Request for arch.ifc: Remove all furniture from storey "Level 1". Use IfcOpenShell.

First a look at what the model holds.

```python
import ifcopenshell
import ifcopenshell.util.element

model = ifcopenshell.open("arch.ifc")
print(model.schema)
storey = next(s for s in model.by_type("IfcBuildingStorey") if s.Name == "Level 1")
furniture = [e for e in ifcopenshell.util.element.get_decomposition(storey) if e.is_a("IfcFurnishingElement")]
seen = {}
for e in furniture:
    element_type = ifcopenshell.util.element.get_type(e)
    name = element_type.Name if element_type not in (None, e) else None
    seen[name] = seen.get(name, 0) + 1
for name, count in sorted(seen.items(), key=str):
    print(count, "x", name)
```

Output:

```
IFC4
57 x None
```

```python
import ifcopenshell
import ifcopenshell.api.root
import ifcopenshell.util.element

model = ifcopenshell.open("arch.ifc")

storey = next(s for s in model.by_type("IfcBuildingStorey") if s.Name == "Level 1")
furniture = [e for e in ifcopenshell.util.element.get_decomposition(storey) if e.is_a("IfcFurnishingElement")]

for e in furniture:
    ifcopenshell.api.root.remove_product(model, product=e)
print(len(furniture), "removed")

model.write("arch_edited.ifc")
```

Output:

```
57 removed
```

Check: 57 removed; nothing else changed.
